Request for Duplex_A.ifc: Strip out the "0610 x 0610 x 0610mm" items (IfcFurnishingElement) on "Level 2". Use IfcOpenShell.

First a look at what the model holds.

```python
import ifcopenshell
import ifcopenshell.util.element

model = ifcopenshell.open("Duplex_A.ifc")
print(model.schema)
storey = next(s for s in model.by_type("IfcBuildingStorey") if s.Name == "Level 2")
furniture = [e for e in ifcopenshell.util.element.get_decomposition(storey) if e.is_a("IfcFurnishingElement")]
seen = {}
for e in furniture:
    element_type = ifcopenshell.util.element.get_type(e)
    name = element_type.Name if element_type not in (None, e) else None
    seen[name] = seen.get(name, 0) + 1
for name, count in sorted(seen.items(), key=str):
    print(count, "x", name)
```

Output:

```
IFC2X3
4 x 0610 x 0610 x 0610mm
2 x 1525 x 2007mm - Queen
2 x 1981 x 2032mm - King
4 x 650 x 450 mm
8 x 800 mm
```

```python
import ifcopenshell
import ifcopenshell.api.root
import ifcopenshell.util.element

model = ifcopenshell.open("Duplex_A.ifc")

storey = next(s for s in model.by_type("IfcBuildingStorey") if s.Name == "Level 2")
furniture = [e for e in ifcopenshell.util.element.get_decomposition(storey) if e.is_a("IfcFurnishingElement")]
targets = [e for e in furniture if (t := ifcopenshell.util.element.get_type(e)) not in (None, e) and t.Name == "0610 x 0610 x 0610mm"]

for e in targets:
    ifcopenshell.api.root.remove_product(model, product=e)
print(len(targets), "removed")

model.write("Duplex_A_rev.ifc")
```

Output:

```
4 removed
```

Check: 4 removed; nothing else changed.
